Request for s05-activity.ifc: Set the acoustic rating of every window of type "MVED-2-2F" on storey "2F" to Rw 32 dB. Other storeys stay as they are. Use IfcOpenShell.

First a look at what the model holds.

```python
import ifcopenshell
import ifcopenshell.util.element

model = ifcopenshell.open("s05-activity.ifc")
print(model.schema)
storey = next(s for s in model.by_type("IfcBuildingStorey") if s.Name == "2F")
windows = [e for e in ifcopenshell.util.element.get_decomposition(storey) if e.is_a("IfcWindow")]
seen = {}
for e in windows:
    element_type = ifcopenshell.util.element.get_type(e)
    key = (element_type.Name if element_type != e and element_type else None, ifcopenshell.util.element.get_pset(e, "Pset_WindowCommon", "AcousticRating"))
    seen[key] = seen.get(key, 0) + 1
for (name, value), count in sorted(seen.items(), key=str):
    print(count, "x", name, "|", value)
```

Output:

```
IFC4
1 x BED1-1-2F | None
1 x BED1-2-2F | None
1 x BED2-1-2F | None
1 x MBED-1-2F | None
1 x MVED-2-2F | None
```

```python
import ifcopenshell
import ifcopenshell.api.pset
import ifcopenshell.util.element

model = ifcopenshell.open("s05-activity.ifc")

storey = next(s for s in model.by_type("IfcBuildingStorey") if s.Name == "2F")
windows = [e for e in ifcopenshell.util.element.get_decomposition(storey) if e.is_a("IfcWindow")]

count = 0
for e in windows:
    element_type = ifcopenshell.util.element.get_type(e)
    if element_type in (None, e) or element_type.Name != "MVED-2-2F":
        continue
    # add_pset returns the element's existing set when there is one.
    pset = ifcopenshell.api.pset.add_pset(model, product=e, name="Pset_WindowCommon")
    ifcopenshell.api.pset.edit_pset(model, pset=pset, properties={"AcousticRating": "Rw 32 dB"})
    count += 1

print(count, "windows updated")

model.write("s05-activity-out.ifc")
```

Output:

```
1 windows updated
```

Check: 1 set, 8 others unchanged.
